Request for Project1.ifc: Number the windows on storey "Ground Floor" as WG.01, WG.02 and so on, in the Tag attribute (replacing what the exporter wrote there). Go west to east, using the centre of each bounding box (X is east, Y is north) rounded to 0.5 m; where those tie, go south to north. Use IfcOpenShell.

First a look at what the model holds.

```python
import ifcopenshell
import ifcopenshell.util.element
import ifcopenshell.util.placement

model = ifcopenshell.open("Project1.ifc")
print(model.schema)
storey = next(s for s in model.by_type("IfcBuildingStorey") if s.Name == "Ground Floor")
windows = [e for e in ifcopenshell.util.element.get_decomposition(storey) if e.is_a("IfcWindow")]
for e in sorted(windows, key=lambda e: e.id()):
    origin = ifcopenshell.util.placement.get_local_placement(e.ObjectPlacement)[:3, 3]
    print(e.id(), e.Tag, e.Name, origin.round(2) + 0.0, sep=" | ")
```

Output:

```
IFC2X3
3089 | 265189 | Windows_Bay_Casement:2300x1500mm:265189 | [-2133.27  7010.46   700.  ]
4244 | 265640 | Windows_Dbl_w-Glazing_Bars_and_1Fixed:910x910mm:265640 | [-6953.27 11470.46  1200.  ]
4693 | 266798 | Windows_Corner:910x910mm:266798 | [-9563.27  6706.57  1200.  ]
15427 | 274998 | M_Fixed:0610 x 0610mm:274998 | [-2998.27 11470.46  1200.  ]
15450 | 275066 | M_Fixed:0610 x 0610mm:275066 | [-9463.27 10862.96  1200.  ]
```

```python
import ifcopenshell
import ifcopenshell.geom
import ifcopenshell.util.element
import ifcopenshell.util.shape

model = ifcopenshell.open("Project1.ifc")
settings = ifcopenshell.geom.settings()
settings.set("use-world-coords", True)


def centre(element):
    shape = ifcopenshell.geom.create_shape(settings, element)
    return ifcopenshell.util.shape.get_bbox_centroid(shape.geometry)


storey = next(s for s in model.by_type("IfcBuildingStorey") if s.Name == "Ground Floor")
windows = [e for e in ifcopenshell.util.element.get_decomposition(storey) if e.is_a("IfcWindow")]

# Insertion points can sit at a corner or the storey origin, so sort by the geometry (in metres).
centres = {e: centre(e) for e in windows}
windows.sort(key=lambda e: (round(centres[e][0] / 0.5), centres[e][1]))

for i, e in enumerate(windows, start=1):
    number = f"WG.{i:02d}"
    e.Tag = number
    print(e.id(), number)

model.write("Project1_v2.ifc")
```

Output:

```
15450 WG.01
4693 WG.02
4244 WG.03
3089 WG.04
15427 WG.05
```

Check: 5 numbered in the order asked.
